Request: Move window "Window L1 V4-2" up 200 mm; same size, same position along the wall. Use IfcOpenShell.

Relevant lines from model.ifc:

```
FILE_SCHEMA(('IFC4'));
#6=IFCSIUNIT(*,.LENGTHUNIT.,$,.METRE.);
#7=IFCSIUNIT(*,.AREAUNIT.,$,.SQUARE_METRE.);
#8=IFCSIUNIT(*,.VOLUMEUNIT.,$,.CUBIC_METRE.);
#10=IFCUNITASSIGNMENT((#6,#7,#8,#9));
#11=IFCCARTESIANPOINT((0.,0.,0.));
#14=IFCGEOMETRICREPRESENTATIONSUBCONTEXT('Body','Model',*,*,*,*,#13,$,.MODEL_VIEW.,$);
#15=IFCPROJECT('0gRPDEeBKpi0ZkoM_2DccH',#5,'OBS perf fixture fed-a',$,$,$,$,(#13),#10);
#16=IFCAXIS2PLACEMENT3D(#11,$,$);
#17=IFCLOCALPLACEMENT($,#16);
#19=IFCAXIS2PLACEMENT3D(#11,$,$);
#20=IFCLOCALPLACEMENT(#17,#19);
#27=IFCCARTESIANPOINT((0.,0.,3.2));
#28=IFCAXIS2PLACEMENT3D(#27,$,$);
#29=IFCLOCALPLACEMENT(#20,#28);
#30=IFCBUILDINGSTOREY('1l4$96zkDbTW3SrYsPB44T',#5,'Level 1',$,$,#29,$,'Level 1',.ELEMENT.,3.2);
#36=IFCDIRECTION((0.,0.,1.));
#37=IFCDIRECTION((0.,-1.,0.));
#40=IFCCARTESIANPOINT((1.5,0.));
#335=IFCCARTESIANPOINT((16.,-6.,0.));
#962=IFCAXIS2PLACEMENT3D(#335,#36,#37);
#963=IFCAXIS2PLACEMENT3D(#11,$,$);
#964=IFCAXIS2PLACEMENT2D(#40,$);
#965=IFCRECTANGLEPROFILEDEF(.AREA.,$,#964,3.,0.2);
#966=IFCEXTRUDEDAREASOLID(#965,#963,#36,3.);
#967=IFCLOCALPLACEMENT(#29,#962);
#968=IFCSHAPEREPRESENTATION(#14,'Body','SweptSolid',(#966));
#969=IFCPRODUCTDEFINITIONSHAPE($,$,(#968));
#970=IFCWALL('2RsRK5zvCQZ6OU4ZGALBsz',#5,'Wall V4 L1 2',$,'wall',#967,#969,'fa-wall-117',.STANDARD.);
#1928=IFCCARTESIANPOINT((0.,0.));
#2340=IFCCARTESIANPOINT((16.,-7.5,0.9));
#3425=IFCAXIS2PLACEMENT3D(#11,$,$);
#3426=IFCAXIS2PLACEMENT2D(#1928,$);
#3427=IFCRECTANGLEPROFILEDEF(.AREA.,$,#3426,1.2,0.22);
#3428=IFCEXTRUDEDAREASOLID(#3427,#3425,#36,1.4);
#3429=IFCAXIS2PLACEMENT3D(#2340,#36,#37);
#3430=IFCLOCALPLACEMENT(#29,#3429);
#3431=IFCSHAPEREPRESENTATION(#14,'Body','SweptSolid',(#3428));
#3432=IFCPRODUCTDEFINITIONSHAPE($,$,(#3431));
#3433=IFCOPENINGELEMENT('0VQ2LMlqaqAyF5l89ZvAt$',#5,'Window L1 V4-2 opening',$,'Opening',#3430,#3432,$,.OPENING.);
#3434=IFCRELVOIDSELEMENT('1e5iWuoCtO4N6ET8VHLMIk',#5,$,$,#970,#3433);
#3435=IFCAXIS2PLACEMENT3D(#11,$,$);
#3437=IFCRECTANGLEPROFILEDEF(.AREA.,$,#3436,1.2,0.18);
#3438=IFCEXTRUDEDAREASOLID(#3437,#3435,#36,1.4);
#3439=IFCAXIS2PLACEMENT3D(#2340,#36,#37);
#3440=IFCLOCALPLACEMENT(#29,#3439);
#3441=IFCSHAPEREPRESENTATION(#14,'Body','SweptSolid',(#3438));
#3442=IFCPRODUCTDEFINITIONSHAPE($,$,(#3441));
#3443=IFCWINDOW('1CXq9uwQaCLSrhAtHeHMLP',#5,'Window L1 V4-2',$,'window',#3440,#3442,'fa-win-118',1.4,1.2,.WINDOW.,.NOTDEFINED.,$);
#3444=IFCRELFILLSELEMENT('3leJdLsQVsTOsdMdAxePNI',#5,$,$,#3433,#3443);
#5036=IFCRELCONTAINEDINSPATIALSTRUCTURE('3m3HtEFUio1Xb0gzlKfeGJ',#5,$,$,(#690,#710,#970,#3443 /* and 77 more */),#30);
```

```python
import numpy as np
import ifcopenshell
import ifcopenshell.api.geometry
import ifcopenshell.util.placement
import ifcopenshell.util.unit

model = ifcopenshell.open("model.ifc")
unit_scale = ifcopenshell.util.unit.calculate_unit_scale(model)

window = model.by_guid("1CXq9uwQaCLSrhAtHeHMLP")
opening = window.FillsVoids[0].RelatingOpeningElement
dz = 0.2

shift = np.array([0.0, 0.0, dz])
# The window is not placed relative to its opening, so move both.
for product in (opening, window):
    matrix = ifcopenshell.util.placement.get_local_placement(product.ObjectPlacement)
    matrix[:3, 3] += shift
    ifcopenshell.api.geometry.edit_object_placement(model, product=product, matrix=matrix, is_si=False)

print(f"moved by {dz * unit_scale:+.3f} m")

model.write("model_edited.ifc")
```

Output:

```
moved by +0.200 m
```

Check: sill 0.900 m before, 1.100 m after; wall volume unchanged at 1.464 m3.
